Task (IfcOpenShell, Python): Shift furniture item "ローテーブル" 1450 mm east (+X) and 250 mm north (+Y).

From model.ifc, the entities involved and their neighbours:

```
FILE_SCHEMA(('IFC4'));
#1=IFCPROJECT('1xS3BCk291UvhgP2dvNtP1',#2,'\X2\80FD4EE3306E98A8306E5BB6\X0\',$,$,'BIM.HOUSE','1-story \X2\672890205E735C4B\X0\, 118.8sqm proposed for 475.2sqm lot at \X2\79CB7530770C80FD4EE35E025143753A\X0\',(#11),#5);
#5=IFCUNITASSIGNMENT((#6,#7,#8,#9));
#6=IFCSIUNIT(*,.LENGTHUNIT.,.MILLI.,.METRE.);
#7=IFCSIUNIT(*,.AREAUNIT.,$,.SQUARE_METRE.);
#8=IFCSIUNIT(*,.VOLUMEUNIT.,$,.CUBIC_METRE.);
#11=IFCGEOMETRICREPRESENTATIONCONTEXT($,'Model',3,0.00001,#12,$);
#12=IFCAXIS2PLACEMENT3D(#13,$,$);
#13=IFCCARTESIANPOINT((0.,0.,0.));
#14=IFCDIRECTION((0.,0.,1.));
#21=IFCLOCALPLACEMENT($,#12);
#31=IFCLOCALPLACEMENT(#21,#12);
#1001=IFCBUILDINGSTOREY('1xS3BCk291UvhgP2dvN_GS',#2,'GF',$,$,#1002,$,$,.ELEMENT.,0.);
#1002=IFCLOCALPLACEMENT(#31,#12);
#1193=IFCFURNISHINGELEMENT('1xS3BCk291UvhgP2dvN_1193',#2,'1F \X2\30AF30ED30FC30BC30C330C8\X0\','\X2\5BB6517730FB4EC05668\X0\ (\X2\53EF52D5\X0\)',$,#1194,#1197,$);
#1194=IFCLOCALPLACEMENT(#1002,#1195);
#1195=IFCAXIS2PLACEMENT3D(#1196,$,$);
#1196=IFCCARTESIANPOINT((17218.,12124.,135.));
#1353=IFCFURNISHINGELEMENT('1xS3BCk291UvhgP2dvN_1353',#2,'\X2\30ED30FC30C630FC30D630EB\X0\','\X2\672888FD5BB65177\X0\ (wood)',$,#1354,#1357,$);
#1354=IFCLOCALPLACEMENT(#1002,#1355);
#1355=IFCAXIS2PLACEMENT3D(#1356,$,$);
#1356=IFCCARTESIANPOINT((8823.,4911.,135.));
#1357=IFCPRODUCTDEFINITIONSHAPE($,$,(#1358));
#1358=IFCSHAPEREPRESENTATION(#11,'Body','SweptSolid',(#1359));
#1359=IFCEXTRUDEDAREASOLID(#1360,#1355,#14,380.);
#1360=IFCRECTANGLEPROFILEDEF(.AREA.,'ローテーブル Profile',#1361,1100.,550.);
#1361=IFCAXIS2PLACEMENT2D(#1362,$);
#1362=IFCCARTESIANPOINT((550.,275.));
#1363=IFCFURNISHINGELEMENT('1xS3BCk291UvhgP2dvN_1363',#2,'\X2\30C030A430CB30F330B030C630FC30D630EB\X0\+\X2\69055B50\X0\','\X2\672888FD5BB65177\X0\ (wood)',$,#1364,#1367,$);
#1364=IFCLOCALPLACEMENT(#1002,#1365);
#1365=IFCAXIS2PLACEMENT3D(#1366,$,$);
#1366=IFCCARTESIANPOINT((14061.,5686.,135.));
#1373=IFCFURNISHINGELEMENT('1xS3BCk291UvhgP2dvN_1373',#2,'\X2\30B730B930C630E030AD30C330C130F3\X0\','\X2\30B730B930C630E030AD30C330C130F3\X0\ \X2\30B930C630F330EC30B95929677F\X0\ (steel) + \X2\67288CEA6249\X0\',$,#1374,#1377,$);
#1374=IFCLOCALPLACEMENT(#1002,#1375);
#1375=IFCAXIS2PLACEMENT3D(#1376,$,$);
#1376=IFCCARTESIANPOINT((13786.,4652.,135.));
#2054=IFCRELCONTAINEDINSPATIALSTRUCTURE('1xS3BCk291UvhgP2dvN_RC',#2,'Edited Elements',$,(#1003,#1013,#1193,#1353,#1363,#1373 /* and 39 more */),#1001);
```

```python
import ifcopenshell
import ifcopenshell.api.geometry
import ifcopenshell.util.placement
import ifcopenshell.util.unit

model = ifcopenshell.open("model.ifc")
unit_scale = ifcopenshell.util.unit.calculate_unit_scale(model)

item = model.by_guid("1xS3BCk291UvhgP2dvN_1353")
matrix = ifcopenshell.util.placement.get_local_placement(item.ObjectPlacement)
matrix[0, 3] += 1.45 / unit_scale
matrix[1, 3] += 0.25 / unit_scale
ifcopenshell.api.geometry.edit_object_placement(model, product=item, matrix=matrix, is_si=False)

print(ifcopenshell.util.placement.get_local_placement(item.ObjectPlacement).round(3) + 0.0)

model.write("model_rev.ifc")
```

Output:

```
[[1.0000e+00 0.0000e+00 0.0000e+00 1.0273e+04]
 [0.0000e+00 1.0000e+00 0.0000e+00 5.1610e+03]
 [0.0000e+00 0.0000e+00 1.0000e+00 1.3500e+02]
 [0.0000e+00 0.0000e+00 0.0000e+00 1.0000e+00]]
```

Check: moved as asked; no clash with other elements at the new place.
